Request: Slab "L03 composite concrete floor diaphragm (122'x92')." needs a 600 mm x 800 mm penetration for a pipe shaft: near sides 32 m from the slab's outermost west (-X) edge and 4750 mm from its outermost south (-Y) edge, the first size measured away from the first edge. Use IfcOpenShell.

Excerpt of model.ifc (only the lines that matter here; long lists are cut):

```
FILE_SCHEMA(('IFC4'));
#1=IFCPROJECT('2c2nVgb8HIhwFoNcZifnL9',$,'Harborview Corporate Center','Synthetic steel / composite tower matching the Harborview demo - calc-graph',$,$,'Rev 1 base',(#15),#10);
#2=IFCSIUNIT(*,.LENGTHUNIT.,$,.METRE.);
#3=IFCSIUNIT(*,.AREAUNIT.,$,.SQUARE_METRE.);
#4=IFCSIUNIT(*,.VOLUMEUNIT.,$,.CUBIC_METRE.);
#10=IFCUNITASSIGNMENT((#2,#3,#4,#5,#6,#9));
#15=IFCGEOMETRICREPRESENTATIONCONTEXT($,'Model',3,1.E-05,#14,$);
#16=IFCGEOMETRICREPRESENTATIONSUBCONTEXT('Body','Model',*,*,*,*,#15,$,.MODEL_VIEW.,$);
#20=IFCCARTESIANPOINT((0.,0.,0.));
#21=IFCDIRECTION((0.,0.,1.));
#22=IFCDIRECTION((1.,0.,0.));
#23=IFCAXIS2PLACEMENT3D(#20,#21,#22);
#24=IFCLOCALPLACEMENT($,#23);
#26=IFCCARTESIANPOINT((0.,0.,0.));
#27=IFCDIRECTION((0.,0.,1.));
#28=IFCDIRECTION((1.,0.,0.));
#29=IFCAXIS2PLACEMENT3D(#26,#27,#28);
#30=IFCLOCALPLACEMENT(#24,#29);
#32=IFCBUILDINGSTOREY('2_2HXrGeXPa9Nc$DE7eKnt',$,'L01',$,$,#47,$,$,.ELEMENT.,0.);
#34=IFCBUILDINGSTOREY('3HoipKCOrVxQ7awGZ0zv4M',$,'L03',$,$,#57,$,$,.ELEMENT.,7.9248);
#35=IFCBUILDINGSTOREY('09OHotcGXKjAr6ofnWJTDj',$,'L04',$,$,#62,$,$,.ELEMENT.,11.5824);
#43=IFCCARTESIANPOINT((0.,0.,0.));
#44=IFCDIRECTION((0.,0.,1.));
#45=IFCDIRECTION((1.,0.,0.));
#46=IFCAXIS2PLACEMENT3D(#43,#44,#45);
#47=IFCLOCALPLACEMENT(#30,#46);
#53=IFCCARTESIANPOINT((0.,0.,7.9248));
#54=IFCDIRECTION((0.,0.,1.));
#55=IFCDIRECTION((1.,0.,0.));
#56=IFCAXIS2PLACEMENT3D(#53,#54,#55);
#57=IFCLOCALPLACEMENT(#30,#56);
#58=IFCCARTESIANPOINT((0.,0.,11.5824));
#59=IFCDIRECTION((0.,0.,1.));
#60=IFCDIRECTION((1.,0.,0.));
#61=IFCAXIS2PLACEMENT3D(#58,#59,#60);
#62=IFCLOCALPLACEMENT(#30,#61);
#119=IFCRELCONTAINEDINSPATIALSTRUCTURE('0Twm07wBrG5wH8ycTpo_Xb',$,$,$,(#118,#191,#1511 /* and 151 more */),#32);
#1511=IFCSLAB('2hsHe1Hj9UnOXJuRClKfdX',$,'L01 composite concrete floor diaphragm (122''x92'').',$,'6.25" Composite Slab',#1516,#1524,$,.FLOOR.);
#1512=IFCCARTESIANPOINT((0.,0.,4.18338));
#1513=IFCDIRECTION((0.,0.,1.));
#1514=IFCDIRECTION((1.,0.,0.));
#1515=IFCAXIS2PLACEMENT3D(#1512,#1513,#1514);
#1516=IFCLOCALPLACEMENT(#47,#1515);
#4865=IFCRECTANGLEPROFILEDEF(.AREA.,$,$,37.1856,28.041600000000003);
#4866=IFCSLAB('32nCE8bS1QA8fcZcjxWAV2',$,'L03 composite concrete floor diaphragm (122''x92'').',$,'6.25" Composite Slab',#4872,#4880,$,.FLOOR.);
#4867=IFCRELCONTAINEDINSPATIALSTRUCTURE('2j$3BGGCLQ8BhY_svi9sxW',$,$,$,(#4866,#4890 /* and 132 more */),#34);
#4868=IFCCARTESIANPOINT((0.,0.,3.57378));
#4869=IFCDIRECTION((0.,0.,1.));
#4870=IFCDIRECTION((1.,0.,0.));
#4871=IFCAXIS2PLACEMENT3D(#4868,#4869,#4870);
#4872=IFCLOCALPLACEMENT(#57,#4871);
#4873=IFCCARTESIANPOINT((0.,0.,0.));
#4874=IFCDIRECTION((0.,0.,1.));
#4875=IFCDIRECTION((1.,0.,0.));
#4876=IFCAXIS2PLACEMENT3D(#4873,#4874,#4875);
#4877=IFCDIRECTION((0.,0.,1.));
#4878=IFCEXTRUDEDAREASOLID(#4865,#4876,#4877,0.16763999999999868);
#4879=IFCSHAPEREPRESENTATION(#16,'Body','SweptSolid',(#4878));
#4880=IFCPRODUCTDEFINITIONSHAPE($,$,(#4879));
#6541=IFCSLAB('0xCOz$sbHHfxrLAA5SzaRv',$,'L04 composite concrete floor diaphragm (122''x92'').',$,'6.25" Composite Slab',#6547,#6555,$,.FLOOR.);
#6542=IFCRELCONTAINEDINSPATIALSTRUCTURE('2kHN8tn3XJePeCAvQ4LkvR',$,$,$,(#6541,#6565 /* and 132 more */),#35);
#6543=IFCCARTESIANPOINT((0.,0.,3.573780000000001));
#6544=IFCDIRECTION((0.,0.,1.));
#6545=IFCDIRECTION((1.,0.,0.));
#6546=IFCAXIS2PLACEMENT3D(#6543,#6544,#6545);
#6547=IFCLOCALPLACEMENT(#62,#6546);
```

```python
import numpy as np
import ifcopenshell
import ifcopenshell.api.feature
import ifcopenshell.api.geometry
import ifcopenshell.api.root
import ifcopenshell.geom
import ifcopenshell.util.placement
import ifcopenshell.util.representation
import ifcopenshell.util.shape
import ifcopenshell.util.unit

model = ifcopenshell.open("model.ifc")
unit_scale = ifcopenshell.util.unit.calculate_unit_scale(model)
settings = ifcopenshell.geom.settings()


def volume(element):
    """Net volume in cubic metres, openings subtracted."""
    shape = ifcopenshell.geom.create_shape(settings, element)
    return ifcopenshell.util.shape.get_volume(shape.geometry)


slab = model.by_guid("32nCE8bS1QA8fcZcjxWAV2")
before = volume(slab)

# Extent in the slab's own axes, in metres. The edges named are its -X and -Y sides.
slab_shape = ifcopenshell.geom.create_shape(settings, slab)
vertices = ifcopenshell.util.shape.get_vertices(slab_shape.geometry)
x_min, y_min, bottom = vertices.min(axis=0)
top = vertices[:, 2].max()

opening = ifcopenshell.api.root.create_entity(model, ifc_class="IfcOpeningElement", name="Pipe shaft opening", predefined_type="OPENING")
context = ifcopenshell.util.representation.get_context(model, "Model", "Body", "MODEL_VIEW")
width, depth = 0.6, 0.8
outline = [(0.0, 0.0), (width, 0.0), (width, depth), (0.0, depth), (0.0, 0.0)]
# Overshoot both faces by 50 mm so the cut is clean.
shape = ifcopenshell.api.geometry.add_slab_representation(
    model, context=context, depth=top - bottom + 0.1, polyline=outline
)
ifcopenshell.api.geometry.assign_representation(model, product=opening, representation=shape)

matrix = ifcopenshell.util.placement.get_local_placement(slab.ObjectPlacement)
matrix[:, 3] = matrix @ np.append(np.array([x_min + 32, y_min + 4.75, bottom - 0.05]) / unit_scale, 1.0)
ifcopenshell.api.geometry.edit_object_placement(model, product=opening, matrix=matrix, is_si=False)
ifcopenshell.api.feature.add_feature(model, feature=opening, element=slab)

after = volume(slab)

print(f"slab volume {before:.3f} -> {after:.3f} m3")

model.write("model_rev.ifc")
```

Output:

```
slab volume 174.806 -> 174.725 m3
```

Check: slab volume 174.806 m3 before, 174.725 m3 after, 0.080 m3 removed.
